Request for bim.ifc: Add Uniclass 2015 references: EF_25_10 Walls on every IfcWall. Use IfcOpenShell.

First a look at what the model holds.

```python
import ifcopenshell

model = ifcopenshell.open("bim.ifc")
print(model.schema)
print("classifications:", [c.Name for c in model.by_type("IfcClassification")])
for ifc_class in ("IfcDoor", "IfcRoof", "IfcStair", "IfcWall", "IfcWindow"):
    print(ifc_class, len(model.by_type(ifc_class)))
```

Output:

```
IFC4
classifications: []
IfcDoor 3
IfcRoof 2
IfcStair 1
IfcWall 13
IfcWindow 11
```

```python
import ifcopenshell
import ifcopenshell.api.classification

model = ifcopenshell.open("bim.ifc")

system = ifcopenshell.api.classification.add_classification(model, classification="Uniclass 2015")

codes = {
    "IfcWall": ("EF_25_10", "Walls"),
}
for ifc_class, (code, name) in codes.items():
    products = model.by_type(ifc_class)
    ifcopenshell.api.classification.add_reference(
        model, products=products, classification=system, identification=code, name=name
    )
    print(code, len(products))

model.write("bim_updated.ifc")
```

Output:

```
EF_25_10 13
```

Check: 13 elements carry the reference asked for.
